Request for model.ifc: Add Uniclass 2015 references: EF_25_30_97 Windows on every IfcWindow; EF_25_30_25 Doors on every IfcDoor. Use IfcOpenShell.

First a look at what the model holds.

```python
import ifcopenshell

model = ifcopenshell.open("model.ifc")
print(model.schema)
print("classifications:", [c.Name for c in model.by_type("IfcClassification")])
for ifc_class in ("IfcDoor", "IfcRoof", "IfcStair", "IfcWall", "IfcWindow"):
    print(ifc_class, len(model.by_type(ifc_class)))
```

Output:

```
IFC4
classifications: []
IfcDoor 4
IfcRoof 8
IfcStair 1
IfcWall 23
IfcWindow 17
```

```python
import ifcopenshell
import ifcopenshell.api.classification

model = ifcopenshell.open("model.ifc")

system = ifcopenshell.api.classification.add_classification(model, classification="Uniclass 2015")

codes = {
    "IfcWindow": ("EF_25_30_97", "Windows"),
    "IfcDoor": ("EF_25_30_25", "Doors"),
}
for ifc_class, (code, name) in codes.items():
    products = model.by_type(ifc_class)
    ifcopenshell.api.classification.add_reference(
        model, products=products, classification=system, identification=code, name=name
    )
    print(code, len(products))

model.write("model_edited.ifc")
```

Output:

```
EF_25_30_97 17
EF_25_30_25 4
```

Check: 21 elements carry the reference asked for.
